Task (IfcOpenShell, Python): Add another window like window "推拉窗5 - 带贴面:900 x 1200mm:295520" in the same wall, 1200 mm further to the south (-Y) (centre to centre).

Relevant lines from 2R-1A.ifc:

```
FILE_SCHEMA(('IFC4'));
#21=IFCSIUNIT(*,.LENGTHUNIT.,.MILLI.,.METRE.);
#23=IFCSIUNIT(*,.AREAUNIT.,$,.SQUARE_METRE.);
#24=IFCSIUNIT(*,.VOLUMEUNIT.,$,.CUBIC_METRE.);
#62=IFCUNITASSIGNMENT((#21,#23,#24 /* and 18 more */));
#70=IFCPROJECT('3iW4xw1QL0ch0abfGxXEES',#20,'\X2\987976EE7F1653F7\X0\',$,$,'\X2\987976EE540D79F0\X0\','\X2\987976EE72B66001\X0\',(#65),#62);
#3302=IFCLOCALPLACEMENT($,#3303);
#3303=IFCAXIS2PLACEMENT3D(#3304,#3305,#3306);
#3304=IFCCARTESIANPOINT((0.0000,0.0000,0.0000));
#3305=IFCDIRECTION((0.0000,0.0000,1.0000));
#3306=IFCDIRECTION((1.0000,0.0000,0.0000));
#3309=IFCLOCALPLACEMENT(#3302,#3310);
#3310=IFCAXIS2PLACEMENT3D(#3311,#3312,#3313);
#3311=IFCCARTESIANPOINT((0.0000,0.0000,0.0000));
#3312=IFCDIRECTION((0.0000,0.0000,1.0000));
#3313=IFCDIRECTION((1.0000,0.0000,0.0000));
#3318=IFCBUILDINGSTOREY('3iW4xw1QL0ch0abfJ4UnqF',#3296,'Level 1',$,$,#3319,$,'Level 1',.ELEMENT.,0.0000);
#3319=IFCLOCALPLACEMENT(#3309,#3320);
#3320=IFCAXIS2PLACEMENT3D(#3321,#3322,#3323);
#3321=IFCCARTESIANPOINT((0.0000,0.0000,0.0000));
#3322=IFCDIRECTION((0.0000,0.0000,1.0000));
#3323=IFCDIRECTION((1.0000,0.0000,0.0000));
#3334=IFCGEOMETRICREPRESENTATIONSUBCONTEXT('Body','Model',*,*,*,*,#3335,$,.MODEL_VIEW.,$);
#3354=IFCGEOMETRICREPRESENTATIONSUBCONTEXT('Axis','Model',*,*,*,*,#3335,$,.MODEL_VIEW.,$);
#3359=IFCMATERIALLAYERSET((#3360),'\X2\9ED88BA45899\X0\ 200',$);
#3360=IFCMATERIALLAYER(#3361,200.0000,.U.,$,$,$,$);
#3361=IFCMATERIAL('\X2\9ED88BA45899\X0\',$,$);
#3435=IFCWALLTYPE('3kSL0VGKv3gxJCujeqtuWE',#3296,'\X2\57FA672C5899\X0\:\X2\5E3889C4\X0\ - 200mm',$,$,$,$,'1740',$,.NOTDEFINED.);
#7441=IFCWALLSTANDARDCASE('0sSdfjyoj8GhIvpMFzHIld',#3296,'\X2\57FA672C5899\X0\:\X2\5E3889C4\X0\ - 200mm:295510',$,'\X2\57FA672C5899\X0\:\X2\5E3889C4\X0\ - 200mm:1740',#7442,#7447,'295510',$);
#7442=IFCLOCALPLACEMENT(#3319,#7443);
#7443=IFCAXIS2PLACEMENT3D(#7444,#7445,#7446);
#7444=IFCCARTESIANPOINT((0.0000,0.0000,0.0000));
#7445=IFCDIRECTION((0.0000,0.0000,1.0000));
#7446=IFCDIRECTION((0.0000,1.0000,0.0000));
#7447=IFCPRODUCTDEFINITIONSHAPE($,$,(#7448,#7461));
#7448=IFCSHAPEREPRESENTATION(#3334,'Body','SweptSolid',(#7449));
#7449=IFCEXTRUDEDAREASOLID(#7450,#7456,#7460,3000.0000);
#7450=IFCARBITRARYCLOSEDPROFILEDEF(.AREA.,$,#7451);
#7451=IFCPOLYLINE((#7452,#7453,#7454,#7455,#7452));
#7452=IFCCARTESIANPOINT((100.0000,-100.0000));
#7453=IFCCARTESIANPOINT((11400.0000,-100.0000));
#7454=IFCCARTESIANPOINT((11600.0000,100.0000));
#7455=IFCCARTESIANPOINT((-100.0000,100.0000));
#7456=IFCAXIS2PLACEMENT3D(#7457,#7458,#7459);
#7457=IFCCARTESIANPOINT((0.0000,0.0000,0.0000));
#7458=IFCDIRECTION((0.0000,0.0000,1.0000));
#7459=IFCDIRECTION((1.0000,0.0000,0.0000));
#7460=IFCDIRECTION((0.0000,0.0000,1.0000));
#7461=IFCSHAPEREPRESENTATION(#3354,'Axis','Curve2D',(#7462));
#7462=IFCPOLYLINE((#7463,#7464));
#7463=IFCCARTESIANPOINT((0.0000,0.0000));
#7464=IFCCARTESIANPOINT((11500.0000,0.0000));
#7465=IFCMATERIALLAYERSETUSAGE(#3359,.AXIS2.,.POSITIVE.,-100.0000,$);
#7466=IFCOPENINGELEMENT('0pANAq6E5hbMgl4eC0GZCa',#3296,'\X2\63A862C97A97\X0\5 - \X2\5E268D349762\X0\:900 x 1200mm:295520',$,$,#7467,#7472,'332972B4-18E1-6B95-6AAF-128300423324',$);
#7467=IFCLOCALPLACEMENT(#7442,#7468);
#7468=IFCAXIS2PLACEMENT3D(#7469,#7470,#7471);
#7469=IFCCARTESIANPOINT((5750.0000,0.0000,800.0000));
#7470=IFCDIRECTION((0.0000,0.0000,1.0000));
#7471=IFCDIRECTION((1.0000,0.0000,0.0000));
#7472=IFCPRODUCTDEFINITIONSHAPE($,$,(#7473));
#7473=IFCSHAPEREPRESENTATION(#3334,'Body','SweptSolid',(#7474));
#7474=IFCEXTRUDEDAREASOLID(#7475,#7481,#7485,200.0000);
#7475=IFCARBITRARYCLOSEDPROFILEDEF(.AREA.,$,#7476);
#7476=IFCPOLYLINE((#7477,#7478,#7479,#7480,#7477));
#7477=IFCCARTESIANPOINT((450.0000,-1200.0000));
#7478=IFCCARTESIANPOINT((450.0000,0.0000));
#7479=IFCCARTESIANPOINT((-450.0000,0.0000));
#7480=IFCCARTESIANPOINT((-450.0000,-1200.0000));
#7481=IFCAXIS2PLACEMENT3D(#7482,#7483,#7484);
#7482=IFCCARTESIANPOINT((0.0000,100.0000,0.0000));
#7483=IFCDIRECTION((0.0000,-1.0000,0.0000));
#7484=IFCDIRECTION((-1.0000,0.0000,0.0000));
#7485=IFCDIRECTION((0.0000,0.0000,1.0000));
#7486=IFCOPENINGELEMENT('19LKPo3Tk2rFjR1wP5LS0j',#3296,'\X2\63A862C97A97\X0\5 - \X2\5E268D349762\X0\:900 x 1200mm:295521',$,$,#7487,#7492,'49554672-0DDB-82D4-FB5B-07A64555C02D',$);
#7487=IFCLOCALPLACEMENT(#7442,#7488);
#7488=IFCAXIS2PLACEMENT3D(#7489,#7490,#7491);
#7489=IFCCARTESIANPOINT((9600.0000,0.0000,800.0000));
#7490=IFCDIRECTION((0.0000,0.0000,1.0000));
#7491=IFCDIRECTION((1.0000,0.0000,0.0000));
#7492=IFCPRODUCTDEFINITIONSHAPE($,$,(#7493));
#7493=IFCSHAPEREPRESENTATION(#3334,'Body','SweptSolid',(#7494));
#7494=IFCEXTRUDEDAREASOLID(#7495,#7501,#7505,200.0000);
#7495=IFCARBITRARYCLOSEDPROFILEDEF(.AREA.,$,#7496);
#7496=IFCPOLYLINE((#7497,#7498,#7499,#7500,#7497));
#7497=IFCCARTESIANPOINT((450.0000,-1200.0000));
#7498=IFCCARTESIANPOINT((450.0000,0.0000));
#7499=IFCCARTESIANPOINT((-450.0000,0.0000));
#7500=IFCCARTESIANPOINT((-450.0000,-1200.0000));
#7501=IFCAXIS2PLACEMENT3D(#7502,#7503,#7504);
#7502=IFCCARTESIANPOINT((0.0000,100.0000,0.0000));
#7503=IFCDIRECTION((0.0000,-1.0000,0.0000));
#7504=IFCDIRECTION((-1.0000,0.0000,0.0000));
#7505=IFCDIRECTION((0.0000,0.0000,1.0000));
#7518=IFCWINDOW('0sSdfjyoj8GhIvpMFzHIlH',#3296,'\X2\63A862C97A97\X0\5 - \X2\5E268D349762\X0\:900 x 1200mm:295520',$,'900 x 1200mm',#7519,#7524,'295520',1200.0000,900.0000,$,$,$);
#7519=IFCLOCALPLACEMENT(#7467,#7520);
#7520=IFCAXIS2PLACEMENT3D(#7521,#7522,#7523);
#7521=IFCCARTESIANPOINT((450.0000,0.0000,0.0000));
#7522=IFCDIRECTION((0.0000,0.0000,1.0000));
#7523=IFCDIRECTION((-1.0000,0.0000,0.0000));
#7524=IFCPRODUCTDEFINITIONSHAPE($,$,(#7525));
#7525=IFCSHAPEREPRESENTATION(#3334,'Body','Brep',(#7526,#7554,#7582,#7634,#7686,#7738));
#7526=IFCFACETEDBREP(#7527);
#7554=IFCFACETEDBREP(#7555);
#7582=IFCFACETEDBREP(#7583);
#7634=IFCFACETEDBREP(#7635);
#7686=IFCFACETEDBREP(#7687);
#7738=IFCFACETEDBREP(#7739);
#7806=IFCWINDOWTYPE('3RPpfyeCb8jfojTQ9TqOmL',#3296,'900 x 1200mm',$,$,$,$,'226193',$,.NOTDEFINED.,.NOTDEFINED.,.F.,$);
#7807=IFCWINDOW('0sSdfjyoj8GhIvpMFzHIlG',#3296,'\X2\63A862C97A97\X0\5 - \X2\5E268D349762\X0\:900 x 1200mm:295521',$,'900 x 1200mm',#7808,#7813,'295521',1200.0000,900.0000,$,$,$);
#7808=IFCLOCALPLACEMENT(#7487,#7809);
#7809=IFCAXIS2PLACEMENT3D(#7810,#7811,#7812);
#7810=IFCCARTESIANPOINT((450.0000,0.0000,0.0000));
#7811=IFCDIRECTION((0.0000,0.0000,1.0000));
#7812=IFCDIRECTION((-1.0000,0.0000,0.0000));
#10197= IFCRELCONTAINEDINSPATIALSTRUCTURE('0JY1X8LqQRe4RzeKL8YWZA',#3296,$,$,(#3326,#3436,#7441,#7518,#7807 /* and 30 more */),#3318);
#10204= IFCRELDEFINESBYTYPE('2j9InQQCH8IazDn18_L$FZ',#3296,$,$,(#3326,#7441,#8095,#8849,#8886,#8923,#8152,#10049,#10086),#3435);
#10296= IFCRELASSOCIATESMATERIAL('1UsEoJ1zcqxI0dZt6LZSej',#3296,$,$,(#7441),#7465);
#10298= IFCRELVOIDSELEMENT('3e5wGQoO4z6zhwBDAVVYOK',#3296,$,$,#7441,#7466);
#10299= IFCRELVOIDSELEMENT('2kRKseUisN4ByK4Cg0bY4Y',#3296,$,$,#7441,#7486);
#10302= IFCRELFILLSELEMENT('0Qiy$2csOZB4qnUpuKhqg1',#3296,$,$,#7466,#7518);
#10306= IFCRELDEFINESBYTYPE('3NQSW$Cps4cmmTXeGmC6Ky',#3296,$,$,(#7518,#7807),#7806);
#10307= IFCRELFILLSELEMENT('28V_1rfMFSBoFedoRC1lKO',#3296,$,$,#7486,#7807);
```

```python
import ifcopenshell
import ifcopenshell.api.feature
import ifcopenshell.api.geometry
import ifcopenshell.api.root
import ifcopenshell.geom
import ifcopenshell.util.element
import ifcopenshell.util.placement
import ifcopenshell.util.shape

model = ifcopenshell.open("2R-1A.ifc")
settings = ifcopenshell.geom.settings()


def volume(element):
    """Net volume in cubic metres, openings subtracted."""
    shape = ifcopenshell.geom.create_shape(settings, element)
    return ifcopenshell.util.shape.get_volume(shape.geometry)


def reuse_history(source, copy):
    """copy_class also copies each property set's owner history, people and application; keep the originals."""
    for rel in copy.IsDefinedBy:
        if rel.is_a("IfcRelDefinesByProperties") and (history := rel.RelatingPropertyDefinition.OwnerHistory):
            rel.RelatingPropertyDefinition.OwnerHistory = source.OwnerHistory
            ifcopenshell.util.element.remove_deep2(model, history)


window = model.by_guid("0sSdfjyoj8GhIvpMFzHIlH")
opening = window.FillsVoids[0].RelatingOpeningElement
wall = opening.VoidsElements[0].RelatingBuildingElement
before = volume(wall)
shift = ifcopenshell.util.placement.get_local_placement(wall.ObjectPlacement)[:3, 0] * -1200.0

# copy_class copies the void relationship, type, container and properties, but no geometry.
new_opening = ifcopenshell.api.root.copy_class(model, product=opening)
new_opening.Representation = ifcopenshell.util.element.copy_deep(
    model, opening.Representation, exclude=["IfcGeometricRepresentationContext", "IfcRepresentationMap"]
)
new_opening.Name = "推拉窗5 - 带贴面:900 x 1200mm"
new_opening.Tag = None
new_window = ifcopenshell.api.root.copy_class(model, product=window)
new_window.Representation = ifcopenshell.util.element.copy_deep(
    model, window.Representation, exclude=["IfcGeometricRepresentationContext", "IfcRepresentationMap"]
)
new_window.Name = "推拉窗5 - 带贴面:900 x 1200mm"
new_window.Tag = None
reuse_history(window, new_window)
ifcopenshell.api.feature.add_filling(model, opening=new_opening, element=new_window)

for old, new in ((opening, new_opening), (window, new_window)):
    matrix = ifcopenshell.util.placement.get_local_placement(old.ObjectPlacement)
    matrix[:3, 3] += shift
    ifcopenshell.api.geometry.edit_object_placement(model, product=new, matrix=matrix, is_si=False)

after = volume(wall)

print(f"wall volume {before:.3f} -> {after:.3f} m3")

model.write("2R-1A_rev.ifc")
```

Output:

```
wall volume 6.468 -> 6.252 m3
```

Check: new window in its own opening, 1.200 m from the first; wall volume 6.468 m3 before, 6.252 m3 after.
